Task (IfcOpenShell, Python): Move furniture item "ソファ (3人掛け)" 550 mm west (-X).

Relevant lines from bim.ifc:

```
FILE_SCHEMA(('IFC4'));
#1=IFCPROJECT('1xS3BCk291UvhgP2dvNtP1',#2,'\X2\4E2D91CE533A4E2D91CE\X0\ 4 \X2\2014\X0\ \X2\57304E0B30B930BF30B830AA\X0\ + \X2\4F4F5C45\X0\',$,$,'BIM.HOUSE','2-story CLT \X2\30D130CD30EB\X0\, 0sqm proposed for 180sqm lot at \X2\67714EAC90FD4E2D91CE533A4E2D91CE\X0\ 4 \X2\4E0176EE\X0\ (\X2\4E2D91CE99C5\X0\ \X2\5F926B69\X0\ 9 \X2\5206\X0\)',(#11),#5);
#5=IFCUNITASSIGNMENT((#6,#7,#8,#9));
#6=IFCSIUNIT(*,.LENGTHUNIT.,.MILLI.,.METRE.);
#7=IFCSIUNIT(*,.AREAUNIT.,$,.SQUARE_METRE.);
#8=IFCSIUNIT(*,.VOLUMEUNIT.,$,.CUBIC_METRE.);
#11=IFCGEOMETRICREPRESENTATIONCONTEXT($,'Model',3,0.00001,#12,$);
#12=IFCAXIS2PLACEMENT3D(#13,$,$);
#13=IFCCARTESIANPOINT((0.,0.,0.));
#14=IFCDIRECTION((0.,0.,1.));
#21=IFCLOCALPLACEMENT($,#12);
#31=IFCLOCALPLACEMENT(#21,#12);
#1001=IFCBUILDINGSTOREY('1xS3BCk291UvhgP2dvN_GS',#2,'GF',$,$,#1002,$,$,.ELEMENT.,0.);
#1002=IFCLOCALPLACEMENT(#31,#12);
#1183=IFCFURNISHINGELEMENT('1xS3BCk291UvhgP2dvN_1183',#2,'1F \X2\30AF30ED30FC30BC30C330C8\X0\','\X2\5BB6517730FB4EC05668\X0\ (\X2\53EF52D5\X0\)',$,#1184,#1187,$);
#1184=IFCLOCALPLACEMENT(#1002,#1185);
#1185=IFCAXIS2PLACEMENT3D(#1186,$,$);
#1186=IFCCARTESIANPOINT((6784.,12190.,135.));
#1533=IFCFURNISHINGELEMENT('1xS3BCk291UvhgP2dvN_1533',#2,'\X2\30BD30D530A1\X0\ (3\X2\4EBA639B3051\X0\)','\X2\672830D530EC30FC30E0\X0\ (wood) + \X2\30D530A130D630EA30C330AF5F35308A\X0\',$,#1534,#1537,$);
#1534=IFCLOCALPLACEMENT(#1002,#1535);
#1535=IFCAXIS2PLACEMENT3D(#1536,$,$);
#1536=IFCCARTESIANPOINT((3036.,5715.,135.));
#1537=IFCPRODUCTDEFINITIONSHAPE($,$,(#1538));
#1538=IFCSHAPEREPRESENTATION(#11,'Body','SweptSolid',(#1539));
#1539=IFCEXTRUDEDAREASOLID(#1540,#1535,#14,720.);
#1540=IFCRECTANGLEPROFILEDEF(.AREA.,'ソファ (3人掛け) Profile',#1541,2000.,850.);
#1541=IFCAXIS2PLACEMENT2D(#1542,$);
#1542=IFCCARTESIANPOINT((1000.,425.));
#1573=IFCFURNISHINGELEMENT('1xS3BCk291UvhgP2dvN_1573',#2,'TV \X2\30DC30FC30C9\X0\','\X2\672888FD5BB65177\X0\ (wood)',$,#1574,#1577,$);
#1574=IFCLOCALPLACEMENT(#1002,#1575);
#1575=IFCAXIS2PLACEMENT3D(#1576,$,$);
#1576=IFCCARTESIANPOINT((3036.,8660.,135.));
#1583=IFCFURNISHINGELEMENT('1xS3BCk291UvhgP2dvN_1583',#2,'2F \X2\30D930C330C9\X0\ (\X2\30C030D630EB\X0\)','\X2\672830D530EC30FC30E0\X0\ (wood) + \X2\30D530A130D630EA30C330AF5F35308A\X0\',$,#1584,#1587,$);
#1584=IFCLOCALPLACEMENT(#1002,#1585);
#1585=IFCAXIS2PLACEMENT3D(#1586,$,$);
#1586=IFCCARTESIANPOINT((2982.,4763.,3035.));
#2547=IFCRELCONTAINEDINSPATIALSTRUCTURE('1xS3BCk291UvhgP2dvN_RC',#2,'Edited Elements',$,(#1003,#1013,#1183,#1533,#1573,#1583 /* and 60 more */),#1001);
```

```python
import ifcopenshell
import ifcopenshell.api.geometry
import ifcopenshell.util.placement
import ifcopenshell.util.unit

model = ifcopenshell.open("bim.ifc")
unit_scale = ifcopenshell.util.unit.calculate_unit_scale(model)

item = model.by_guid("1xS3BCk291UvhgP2dvN_1533")
matrix = ifcopenshell.util.placement.get_local_placement(item.ObjectPlacement)
matrix[0, 3] -= 0.55 / unit_scale
ifcopenshell.api.geometry.edit_object_placement(model, product=item, matrix=matrix, is_si=False)

print(ifcopenshell.util.placement.get_local_placement(item.ObjectPlacement).round(3) + 0.0)

model.write("bim-out.ifc")
```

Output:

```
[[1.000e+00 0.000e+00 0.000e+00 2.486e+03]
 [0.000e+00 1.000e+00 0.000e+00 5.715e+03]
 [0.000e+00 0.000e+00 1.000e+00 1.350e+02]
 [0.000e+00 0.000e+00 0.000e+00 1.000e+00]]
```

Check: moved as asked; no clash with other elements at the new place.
